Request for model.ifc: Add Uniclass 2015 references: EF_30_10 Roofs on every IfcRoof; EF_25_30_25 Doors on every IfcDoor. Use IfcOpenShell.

First a look at what the model holds.

```python
import ifcopenshell

model = ifcopenshell.open("model.ifc")
print(model.schema)
print("classifications:", [c.Name for c in model.by_type("IfcClassification")])
for ifc_class in ("IfcDoor", "IfcRoof", "IfcStair", "IfcWall", "IfcWindow"):
    print(ifc_class, len(model.by_type(ifc_class)))
```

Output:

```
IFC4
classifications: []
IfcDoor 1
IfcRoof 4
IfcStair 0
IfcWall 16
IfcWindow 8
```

```python
import ifcopenshell
import ifcopenshell.api.classification

model = ifcopenshell.open("model.ifc")

system = ifcopenshell.api.classification.add_classification(model, classification="Uniclass 2015")

codes = {
    "IfcRoof": ("EF_30_10", "Roofs"),
    "IfcDoor": ("EF_25_30_25", "Doors"),
}
for ifc_class, (code, name) in codes.items():
    products = model.by_type(ifc_class)
    ifcopenshell.api.classification.add_reference(
        model, products=products, classification=system, identification=code, name=name
    )
    print(code, len(products))

model.write("model_v2.ifc")
```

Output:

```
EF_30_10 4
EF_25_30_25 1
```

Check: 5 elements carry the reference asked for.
